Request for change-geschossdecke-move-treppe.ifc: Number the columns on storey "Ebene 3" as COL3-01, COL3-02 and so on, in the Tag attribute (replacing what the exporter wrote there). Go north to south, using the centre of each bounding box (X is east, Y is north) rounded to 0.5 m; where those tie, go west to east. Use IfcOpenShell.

First a look at what the model holds.

```python
import ifcopenshell
import ifcopenshell.util.element
import ifcopenshell.util.placement

model = ifcopenshell.open("change-geschossdecke-move-treppe.ifc")
print(model.schema)
storey = next(s for s in model.by_type("IfcBuildingStorey") if s.Name == "Ebene 3")
columns = [e for e in ifcopenshell.util.element.get_decomposition(storey) if e.is_a("IfcColumn")]
for e in sorted(columns, key=lambda e: e.id()):
    origin = ifcopenshell.util.placement.get_local_placement(e.ObjectPlacement)[:3, 3]
    print(e.id(), e.Tag, e.Name, origin.round(2) + 0.0, sep=" | ")
```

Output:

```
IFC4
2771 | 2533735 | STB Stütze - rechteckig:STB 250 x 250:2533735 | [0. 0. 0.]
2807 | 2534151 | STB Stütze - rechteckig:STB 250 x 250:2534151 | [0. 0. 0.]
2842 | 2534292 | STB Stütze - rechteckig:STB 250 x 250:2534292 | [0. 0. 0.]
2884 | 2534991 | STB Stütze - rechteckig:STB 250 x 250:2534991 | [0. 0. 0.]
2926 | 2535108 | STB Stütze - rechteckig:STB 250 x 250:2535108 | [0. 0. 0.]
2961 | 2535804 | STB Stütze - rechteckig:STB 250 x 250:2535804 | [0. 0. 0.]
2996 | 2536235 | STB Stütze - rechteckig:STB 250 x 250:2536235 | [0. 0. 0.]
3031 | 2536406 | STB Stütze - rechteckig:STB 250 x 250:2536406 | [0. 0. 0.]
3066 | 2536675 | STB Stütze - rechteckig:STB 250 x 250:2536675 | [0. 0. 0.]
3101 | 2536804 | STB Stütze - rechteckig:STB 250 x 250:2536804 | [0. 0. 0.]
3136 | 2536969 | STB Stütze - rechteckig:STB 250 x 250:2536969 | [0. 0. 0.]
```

```python
import ifcopenshell
import ifcopenshell.geom
import ifcopenshell.util.element
import ifcopenshell.util.shape

model = ifcopenshell.open("change-geschossdecke-move-treppe.ifc")
settings = ifcopenshell.geom.settings()
settings.set("use-world-coords", True)


def centre(element):
    shape = ifcopenshell.geom.create_shape(settings, element)
    return ifcopenshell.util.shape.get_bbox_centroid(shape.geometry)


storey = next(s for s in model.by_type("IfcBuildingStorey") if s.Name == "Ebene 3")
columns = [e for e in ifcopenshell.util.element.get_decomposition(storey) if e.is_a("IfcColumn")]

# Insertion points can sit at a corner or the storey origin, so sort by the geometry (in metres).
centres = {e: centre(e) for e in columns}
columns.sort(key=lambda e: (-round(centres[e][1] / 0.5), centres[e][0]))

for i, e in enumerate(columns, start=1):
    number = f"COL3-{i:02d}"
    e.Tag = number
    print(e.id(), number)

model.write("change-geschossdecke-move-treppe_v2.ifc")
```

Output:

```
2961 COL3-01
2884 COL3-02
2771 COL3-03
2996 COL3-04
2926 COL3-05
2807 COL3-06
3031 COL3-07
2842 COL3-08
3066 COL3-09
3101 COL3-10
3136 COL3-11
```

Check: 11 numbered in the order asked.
